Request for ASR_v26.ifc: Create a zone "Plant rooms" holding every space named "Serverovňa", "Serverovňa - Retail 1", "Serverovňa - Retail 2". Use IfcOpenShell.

First a look at what the model holds.

```python
import ifcopenshell

model = ifcopenshell.open("ASR_v26.ifc")
print(model.schema)
seen = {}
for space in model.by_type("IfcSpace"):
    seen[space.LongName] = seen.get(space.LongName, 0) + 1
for name, count in sorted(seen.items(), key=str):
    print(count, "x", name)
print("zones:", [z.Name for z in model.by_type("IfcZone")][:20])
```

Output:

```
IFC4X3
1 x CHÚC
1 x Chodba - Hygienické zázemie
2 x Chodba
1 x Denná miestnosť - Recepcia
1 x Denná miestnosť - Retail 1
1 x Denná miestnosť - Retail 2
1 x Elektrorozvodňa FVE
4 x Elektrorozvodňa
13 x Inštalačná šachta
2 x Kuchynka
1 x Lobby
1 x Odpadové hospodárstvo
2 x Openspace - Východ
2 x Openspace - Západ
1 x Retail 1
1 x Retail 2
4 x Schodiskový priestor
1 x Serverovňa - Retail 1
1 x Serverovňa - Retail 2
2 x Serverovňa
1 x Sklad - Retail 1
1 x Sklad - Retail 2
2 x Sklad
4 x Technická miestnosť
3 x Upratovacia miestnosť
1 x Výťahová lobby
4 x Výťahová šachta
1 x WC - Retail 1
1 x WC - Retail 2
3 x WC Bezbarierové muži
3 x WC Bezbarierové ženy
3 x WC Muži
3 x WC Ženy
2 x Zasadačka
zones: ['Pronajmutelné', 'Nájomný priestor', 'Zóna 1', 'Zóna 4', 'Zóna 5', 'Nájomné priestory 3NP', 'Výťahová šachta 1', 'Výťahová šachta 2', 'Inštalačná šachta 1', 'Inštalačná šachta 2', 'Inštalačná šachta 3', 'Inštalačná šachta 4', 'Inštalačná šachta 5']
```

```python
import ifcopenshell
import ifcopenshell.api.group
import ifcopenshell.api.root

model = ifcopenshell.open("ASR_v26.ifc")

names = {"Serverovňa", "Serverovňa - Retail 1", "Serverovňa - Retail 2"}
spaces = [s for s in model.by_type("IfcSpace") if s.LongName in names]

zone = ifcopenshell.api.root.create_entity(model, ifc_class="IfcZone", name="Plant rooms")
ifcopenshell.api.group.assign_group(model, products=spaces, group=zone)
print(len(spaces), "spaces in", zone.Name)

model.write("ASR_v26_updated.ifc")
```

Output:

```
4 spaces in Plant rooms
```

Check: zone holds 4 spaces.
